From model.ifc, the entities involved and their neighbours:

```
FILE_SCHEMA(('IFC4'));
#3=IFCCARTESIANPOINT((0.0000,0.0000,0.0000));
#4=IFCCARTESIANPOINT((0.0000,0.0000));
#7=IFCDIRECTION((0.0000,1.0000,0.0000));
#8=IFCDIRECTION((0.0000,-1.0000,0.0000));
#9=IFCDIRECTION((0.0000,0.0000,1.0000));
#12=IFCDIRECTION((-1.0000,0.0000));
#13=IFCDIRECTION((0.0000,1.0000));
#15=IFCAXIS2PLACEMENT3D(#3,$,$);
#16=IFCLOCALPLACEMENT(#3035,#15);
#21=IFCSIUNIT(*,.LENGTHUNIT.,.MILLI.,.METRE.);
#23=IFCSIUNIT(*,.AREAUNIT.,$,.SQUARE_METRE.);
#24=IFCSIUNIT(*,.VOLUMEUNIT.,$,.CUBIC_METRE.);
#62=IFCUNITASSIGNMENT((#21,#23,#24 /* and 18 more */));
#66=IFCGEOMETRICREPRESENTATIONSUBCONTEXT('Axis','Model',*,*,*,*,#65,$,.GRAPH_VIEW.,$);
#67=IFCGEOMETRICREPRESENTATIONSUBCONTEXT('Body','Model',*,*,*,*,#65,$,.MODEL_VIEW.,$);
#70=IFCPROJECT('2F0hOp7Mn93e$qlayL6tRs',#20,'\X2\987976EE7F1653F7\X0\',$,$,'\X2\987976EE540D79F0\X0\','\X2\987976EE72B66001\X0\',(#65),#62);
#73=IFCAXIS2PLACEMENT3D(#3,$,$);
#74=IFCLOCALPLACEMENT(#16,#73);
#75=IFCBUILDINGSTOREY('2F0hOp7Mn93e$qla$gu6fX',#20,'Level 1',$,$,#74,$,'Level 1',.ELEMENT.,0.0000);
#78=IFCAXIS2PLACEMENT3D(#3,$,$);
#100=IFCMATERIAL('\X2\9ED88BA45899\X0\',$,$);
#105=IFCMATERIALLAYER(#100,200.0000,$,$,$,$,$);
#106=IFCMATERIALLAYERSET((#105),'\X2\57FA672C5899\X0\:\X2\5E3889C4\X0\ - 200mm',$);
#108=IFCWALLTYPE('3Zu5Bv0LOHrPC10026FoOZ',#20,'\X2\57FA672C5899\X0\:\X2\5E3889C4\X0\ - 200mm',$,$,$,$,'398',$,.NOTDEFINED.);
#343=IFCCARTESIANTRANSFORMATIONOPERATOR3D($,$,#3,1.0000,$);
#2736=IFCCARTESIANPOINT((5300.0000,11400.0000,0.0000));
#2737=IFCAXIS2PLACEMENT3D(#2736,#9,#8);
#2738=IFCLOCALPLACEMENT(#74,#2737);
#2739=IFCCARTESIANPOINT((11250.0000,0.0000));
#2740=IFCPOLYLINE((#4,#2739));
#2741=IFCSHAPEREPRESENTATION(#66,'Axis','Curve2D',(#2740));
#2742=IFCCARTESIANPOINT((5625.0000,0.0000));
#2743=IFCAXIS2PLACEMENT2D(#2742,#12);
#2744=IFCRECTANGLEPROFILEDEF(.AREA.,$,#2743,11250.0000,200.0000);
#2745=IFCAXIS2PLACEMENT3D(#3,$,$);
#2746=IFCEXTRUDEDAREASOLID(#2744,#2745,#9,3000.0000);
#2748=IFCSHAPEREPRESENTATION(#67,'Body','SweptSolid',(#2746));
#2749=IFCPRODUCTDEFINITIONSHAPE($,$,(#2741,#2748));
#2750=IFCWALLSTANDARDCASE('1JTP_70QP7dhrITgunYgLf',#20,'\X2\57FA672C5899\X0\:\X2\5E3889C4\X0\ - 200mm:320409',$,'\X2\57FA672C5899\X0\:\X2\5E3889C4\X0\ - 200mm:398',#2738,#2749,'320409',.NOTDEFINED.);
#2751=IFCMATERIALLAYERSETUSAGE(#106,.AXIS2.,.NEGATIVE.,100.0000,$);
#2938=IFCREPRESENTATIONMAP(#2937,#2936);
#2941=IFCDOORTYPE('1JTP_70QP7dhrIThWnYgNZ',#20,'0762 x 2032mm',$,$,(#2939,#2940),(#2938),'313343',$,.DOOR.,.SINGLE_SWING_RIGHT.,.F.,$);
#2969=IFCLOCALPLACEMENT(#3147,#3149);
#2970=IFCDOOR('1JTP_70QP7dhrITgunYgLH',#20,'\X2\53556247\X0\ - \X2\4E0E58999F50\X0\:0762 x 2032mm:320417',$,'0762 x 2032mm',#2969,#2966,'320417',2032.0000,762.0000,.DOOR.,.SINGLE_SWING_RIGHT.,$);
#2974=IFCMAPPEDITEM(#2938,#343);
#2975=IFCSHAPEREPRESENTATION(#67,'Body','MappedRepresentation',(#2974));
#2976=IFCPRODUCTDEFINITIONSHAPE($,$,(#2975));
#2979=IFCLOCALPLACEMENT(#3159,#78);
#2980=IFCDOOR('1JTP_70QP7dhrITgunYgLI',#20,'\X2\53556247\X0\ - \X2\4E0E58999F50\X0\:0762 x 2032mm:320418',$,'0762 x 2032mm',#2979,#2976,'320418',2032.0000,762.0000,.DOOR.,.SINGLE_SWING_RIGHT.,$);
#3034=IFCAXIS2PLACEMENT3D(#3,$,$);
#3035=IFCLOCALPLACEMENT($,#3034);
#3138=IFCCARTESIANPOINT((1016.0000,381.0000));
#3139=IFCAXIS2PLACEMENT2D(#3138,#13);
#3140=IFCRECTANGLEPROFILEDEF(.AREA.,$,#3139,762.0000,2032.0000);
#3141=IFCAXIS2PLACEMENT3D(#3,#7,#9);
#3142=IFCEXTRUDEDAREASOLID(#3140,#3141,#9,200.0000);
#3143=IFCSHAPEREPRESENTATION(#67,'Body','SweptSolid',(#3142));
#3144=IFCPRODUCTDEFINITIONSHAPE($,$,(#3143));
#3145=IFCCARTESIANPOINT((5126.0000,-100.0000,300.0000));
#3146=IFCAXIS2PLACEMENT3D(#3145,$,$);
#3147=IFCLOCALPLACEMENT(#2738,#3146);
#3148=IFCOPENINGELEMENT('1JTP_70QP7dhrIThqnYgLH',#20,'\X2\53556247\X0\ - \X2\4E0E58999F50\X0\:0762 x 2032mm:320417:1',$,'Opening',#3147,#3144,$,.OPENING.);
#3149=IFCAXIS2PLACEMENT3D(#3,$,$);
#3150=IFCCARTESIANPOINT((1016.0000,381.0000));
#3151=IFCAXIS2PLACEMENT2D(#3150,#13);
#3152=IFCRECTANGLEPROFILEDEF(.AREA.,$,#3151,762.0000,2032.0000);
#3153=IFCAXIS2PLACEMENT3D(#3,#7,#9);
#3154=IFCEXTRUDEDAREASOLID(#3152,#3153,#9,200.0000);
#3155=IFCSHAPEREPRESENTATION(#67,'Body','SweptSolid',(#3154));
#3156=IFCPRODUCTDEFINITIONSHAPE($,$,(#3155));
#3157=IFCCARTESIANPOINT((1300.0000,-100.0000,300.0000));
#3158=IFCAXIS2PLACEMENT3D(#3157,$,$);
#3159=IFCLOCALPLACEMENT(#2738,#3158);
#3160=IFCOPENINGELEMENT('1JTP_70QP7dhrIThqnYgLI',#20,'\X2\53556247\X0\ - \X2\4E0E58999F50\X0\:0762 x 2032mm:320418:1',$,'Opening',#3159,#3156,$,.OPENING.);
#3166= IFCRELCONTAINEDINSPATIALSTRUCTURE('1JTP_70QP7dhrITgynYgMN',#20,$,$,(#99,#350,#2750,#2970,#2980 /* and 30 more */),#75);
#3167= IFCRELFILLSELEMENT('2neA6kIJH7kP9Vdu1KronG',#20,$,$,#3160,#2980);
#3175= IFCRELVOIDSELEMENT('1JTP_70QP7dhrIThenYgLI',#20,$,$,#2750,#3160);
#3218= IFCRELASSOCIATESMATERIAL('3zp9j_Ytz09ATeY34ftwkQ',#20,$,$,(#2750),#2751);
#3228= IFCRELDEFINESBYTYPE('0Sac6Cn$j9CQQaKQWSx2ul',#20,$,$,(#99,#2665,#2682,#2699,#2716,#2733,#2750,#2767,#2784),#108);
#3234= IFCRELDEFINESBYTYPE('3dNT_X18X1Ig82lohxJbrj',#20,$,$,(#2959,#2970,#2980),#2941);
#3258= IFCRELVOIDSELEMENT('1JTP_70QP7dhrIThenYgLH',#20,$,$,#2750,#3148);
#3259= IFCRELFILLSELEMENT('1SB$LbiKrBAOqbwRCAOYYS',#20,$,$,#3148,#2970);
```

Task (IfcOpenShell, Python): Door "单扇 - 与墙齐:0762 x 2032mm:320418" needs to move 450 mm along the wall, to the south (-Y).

```python
import ifcopenshell
import ifcopenshell.api.geometry
import ifcopenshell.util.placement
import ifcopenshell.util.unit

model = ifcopenshell.open("model.ifc")
unit_scale = ifcopenshell.util.unit.calculate_unit_scale(model)

door = model.by_guid("1JTP_70QP7dhrITgunYgLI")
opening = door.FillsVoids[0].RelatingOpeningElement
wall = opening.VoidsElements[0].RelatingBuildingElement

wall_matrix = ifcopenshell.util.placement.get_local_placement(wall.ObjectPlacement)
shift = wall_matrix[:3, 0] * 0.45 / unit_scale
before = ifcopenshell.util.placement.get_local_placement(door.ObjectPlacement)[:3, 3].copy()

# The door is placed relative to its opening, so it follows when the opening moves.
matrix = ifcopenshell.util.placement.get_local_placement(opening.ObjectPlacement)
matrix[:3, 3] += shift
ifcopenshell.api.geometry.edit_object_placement(
    model, product=opening, matrix=matrix, is_si=False, should_transform_children=True
)

after = ifcopenshell.util.placement.get_local_placement(door.ObjectPlacement)[:3, 3]
print("door moved by", (after - before).round(3) + 0.0)

model.write("model-out.ifc")
```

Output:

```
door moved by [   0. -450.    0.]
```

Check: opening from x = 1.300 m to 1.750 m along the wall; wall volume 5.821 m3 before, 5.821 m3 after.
